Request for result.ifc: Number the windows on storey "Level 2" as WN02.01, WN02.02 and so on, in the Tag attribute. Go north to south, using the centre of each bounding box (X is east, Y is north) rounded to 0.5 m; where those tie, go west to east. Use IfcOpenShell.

First a look at what the model holds.

```python
import ifcopenshell
import ifcopenshell.util.element
import ifcopenshell.util.placement

model = ifcopenshell.open("result.ifc")
print(model.schema)
storey = next(s for s in model.by_type("IfcBuildingStorey") if s.Name == "Level 2")
windows = [e for e in ifcopenshell.util.element.get_decomposition(storey) if e.is_a("IfcWindow")]
for e in sorted(windows, key=lambda e: e.id()):
    origin = ifcopenshell.util.placement.get_local_placement(e.ObjectPlacement)[:3, 3]
    print(e.id(), e.Tag, e.Name, origin.round(2) + 0.0, sep=" | ")
```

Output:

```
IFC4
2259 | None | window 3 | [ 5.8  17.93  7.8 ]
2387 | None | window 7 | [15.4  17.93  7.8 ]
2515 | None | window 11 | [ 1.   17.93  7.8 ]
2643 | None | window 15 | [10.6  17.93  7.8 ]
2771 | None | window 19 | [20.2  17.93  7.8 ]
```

```python
import ifcopenshell
import ifcopenshell.geom
import ifcopenshell.util.element
import ifcopenshell.util.shape

model = ifcopenshell.open("result.ifc")
settings = ifcopenshell.geom.settings()
settings.set("use-world-coords", True)


def centre(element):
    shape = ifcopenshell.geom.create_shape(settings, element)
    return ifcopenshell.util.shape.get_bbox_centroid(shape.geometry)


storey = next(s for s in model.by_type("IfcBuildingStorey") if s.Name == "Level 2")
windows = [e for e in ifcopenshell.util.element.get_decomposition(storey) if e.is_a("IfcWindow")]

# Insertion points can sit at a corner or the storey origin, so sort by the geometry (in metres).
centres = {e: centre(e) for e in windows}
windows.sort(key=lambda e: (-round(centres[e][1] / 0.5), centres[e][0]))

for i, e in enumerate(windows, start=1):
    number = f"WN02.{i:02d}"
    e.Tag = number
    print(e.id(), number)

model.write("result_edited.ifc")
```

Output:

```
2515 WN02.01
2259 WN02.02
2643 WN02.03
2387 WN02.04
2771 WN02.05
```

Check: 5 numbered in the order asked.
